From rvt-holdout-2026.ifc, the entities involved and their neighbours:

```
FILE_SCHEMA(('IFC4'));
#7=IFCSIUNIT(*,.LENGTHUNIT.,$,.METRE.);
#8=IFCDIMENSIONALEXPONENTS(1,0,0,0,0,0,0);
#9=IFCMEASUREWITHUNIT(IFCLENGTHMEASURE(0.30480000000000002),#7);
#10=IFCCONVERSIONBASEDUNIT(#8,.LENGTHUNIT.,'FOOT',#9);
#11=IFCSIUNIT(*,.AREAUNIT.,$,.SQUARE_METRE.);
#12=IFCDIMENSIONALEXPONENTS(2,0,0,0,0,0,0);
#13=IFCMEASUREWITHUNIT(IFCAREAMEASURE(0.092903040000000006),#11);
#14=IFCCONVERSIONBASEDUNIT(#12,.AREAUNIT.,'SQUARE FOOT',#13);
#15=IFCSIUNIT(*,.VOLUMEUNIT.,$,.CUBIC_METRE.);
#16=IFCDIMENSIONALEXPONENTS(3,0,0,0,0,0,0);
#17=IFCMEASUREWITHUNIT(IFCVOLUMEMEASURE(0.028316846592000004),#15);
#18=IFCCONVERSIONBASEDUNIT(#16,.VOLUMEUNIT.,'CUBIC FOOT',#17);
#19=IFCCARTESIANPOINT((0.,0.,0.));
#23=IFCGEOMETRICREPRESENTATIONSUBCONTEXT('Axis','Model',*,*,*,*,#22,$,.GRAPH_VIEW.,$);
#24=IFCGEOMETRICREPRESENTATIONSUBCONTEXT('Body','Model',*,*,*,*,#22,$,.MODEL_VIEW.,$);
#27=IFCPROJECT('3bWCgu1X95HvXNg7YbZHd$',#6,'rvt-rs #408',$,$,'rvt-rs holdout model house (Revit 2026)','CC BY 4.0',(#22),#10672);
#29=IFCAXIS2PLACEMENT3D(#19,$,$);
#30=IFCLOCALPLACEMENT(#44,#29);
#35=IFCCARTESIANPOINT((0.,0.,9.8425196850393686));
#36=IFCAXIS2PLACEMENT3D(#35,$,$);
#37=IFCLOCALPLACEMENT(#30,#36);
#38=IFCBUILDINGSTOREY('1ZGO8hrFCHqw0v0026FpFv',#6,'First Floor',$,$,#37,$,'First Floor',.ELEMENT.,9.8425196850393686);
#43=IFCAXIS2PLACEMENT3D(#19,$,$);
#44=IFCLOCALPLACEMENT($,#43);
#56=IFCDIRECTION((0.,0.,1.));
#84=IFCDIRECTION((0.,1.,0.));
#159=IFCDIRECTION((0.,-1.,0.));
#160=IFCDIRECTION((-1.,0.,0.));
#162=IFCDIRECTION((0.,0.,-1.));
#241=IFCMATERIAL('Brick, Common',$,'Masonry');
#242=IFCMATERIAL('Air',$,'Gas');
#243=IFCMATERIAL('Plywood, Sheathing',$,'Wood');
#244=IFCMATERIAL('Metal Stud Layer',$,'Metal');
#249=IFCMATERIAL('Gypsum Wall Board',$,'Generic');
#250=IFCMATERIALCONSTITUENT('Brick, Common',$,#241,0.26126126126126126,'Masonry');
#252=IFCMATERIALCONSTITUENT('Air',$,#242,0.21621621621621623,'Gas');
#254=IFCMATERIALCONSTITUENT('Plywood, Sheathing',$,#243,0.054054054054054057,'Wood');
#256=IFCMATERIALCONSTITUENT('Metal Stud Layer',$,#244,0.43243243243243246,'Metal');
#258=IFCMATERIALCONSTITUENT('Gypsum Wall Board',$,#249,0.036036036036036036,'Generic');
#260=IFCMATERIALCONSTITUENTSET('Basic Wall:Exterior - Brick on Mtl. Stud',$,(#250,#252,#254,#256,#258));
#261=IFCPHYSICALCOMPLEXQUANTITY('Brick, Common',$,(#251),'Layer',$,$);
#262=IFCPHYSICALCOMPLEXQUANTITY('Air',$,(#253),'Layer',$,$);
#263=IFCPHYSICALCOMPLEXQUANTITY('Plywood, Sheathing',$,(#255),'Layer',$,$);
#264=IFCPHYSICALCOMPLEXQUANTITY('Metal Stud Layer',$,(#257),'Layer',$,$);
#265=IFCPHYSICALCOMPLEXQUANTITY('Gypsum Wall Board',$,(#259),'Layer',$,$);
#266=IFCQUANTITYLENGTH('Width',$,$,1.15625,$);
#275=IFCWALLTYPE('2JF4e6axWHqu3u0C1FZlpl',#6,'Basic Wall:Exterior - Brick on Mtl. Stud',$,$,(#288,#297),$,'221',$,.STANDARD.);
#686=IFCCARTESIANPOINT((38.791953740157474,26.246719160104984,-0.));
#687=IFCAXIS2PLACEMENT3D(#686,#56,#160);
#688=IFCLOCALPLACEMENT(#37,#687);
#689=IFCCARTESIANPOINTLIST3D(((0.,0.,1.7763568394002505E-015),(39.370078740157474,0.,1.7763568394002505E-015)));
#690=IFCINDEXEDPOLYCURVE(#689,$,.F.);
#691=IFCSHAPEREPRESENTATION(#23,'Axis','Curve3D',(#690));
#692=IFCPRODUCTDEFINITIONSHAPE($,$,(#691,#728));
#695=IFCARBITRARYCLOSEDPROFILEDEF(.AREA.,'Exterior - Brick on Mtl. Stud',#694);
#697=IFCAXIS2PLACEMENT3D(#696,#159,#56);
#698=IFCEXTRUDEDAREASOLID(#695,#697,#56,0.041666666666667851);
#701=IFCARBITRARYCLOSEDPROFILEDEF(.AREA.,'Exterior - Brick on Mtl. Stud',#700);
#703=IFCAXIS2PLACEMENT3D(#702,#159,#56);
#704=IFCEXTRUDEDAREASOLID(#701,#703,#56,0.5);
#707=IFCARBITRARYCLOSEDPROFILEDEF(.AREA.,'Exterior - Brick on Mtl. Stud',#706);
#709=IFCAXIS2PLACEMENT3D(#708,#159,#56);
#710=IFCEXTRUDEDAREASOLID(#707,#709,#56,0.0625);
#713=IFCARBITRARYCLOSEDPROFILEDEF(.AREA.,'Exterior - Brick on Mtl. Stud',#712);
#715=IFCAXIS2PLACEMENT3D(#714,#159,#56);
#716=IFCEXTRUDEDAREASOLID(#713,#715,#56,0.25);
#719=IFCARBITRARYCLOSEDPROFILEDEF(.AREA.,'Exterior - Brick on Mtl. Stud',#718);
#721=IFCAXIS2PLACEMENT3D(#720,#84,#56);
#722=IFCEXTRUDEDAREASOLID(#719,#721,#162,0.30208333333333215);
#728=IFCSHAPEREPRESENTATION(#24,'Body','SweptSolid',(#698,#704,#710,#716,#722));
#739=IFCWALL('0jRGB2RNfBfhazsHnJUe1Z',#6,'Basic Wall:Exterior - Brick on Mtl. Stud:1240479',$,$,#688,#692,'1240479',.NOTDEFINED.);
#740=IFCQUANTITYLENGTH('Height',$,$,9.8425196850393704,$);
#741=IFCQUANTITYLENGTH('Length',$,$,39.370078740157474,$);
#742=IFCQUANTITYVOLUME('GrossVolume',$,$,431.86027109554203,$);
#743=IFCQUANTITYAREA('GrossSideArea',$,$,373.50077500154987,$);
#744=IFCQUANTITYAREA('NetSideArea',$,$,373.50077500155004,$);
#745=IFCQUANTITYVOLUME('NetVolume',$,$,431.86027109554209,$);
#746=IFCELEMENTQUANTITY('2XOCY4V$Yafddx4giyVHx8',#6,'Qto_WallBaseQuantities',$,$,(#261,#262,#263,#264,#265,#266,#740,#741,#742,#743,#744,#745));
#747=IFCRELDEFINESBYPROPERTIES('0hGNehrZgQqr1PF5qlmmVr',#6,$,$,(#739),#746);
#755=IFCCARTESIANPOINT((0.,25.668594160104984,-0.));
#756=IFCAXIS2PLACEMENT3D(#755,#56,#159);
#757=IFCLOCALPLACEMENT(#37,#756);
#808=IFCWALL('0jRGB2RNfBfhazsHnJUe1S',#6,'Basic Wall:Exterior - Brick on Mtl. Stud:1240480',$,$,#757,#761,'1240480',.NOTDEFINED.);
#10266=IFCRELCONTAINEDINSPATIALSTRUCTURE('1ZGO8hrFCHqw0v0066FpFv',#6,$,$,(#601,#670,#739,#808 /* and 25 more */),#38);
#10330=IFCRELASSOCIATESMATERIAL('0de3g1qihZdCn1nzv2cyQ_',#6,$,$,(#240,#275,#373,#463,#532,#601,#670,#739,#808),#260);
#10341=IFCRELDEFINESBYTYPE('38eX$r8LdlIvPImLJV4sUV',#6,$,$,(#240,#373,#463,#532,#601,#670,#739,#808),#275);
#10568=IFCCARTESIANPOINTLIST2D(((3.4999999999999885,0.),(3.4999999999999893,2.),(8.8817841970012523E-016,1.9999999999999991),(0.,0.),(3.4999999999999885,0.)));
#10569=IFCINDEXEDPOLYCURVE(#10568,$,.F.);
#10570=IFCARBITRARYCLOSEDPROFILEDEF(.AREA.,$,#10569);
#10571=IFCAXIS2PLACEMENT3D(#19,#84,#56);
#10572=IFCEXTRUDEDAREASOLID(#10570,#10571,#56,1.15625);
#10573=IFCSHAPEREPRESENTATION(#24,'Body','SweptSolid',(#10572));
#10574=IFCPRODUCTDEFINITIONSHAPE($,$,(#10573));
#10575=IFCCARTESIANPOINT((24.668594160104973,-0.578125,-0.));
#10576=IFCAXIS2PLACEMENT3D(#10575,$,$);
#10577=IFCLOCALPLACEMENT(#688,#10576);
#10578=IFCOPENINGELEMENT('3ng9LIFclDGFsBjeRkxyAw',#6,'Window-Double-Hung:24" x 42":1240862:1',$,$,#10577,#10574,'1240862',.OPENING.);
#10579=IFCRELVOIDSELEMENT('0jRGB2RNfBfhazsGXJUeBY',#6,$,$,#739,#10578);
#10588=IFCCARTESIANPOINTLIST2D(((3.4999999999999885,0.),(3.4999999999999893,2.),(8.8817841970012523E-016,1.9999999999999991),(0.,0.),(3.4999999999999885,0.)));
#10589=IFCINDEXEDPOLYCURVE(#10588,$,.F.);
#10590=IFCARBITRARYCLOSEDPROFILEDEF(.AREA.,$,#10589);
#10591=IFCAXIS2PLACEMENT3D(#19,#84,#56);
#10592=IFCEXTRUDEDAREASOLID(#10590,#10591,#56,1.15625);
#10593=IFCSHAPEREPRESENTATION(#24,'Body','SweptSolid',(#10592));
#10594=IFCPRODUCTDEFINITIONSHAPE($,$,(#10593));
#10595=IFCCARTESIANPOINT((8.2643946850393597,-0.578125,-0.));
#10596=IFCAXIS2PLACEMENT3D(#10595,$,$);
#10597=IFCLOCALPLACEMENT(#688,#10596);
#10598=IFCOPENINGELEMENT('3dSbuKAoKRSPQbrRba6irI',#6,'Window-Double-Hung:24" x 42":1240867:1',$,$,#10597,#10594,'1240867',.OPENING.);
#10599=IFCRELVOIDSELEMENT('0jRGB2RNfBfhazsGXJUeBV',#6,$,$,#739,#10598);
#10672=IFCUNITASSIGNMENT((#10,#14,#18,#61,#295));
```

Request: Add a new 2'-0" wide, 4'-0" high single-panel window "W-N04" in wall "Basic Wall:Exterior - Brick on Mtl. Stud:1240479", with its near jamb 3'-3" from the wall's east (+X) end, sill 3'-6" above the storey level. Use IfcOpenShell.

```python
import numpy as np
import ifcopenshell
import ifcopenshell.api.feature
import ifcopenshell.api.geometry
import ifcopenshell.api.pset
import ifcopenshell.api.root
import ifcopenshell.api.spatial
import ifcopenshell.geom
import ifcopenshell.util.element
import ifcopenshell.util.placement
import ifcopenshell.util.representation
import ifcopenshell.util.shape
import ifcopenshell.util.unit

model = ifcopenshell.open("rvt-holdout-2026.ifc")
unit_scale = ifcopenshell.util.unit.calculate_unit_scale(model)
area_scale = ifcopenshell.util.unit.calculate_unit_scale(model, "AREAUNIT")
volume_scale = ifcopenshell.util.unit.calculate_unit_scale(model, "VOLUMEUNIT")
settings = ifcopenshell.geom.settings()


def volume(element):
    """Net volume in cubic metres, openings subtracted."""
    shape = ifcopenshell.geom.create_shape(settings, element)
    return ifcopenshell.util.shape.get_volume(shape.geometry)


wall = model.by_guid("0jRGB2RNfBfhazsHnJUe1Z")
storey = ifcopenshell.util.element.get_container(wall, ifc_class="IfcBuildingStorey")
context = ifcopenshell.util.representation.get_context(model, "Model", "Body", "MODEL_VIEW")
before = volume(wall)

width, height, from_end, sill = 0.6096, 1.2192, 0.9906, 1.0668  # metres

# The wall runs along its own X axis, and the end named is its -X end.
wall_shape = ifcopenshell.geom.create_shape(settings, wall)
x, y, z = ifcopenshell.util.shape.get_vertices(wall_shape.geometry).T
start = x.min() + from_end
face, thickness = float(y.min()), float(y.max() - y.min())
wall_matrix = ifcopenshell.util.placement.get_local_placement(wall.ObjectPlacement)
level = ifcopenshell.util.placement.get_local_placement(storey.ObjectPlacement)[2, 3]


def in_wall(x, y):
    """Placement at x, y metres in the wall's axes, at sill height."""
    matrix = wall_matrix.copy()
    matrix[:, 3] = wall_matrix @ np.array([x / unit_scale, y / unit_scale, 0.0, 1.0])
    matrix[2, 3] = level + sill / unit_scale
    return matrix


# Opening: a box that overshoots both wall faces by 50 mm.
opening = ifcopenshell.api.root.create_entity(model, ifc_class="IfcOpeningElement", predefined_type="OPENING")
box = ifcopenshell.api.geometry.add_wall_representation(
    model, context=context, length=width, height=height, thickness=thickness + 0.1
)
ifcopenshell.api.geometry.assign_representation(model, product=opening, representation=box)
ifcopenshell.api.geometry.edit_object_placement(model, product=opening, matrix=in_wall(start, face - 0.05), is_si=False)
ifcopenshell.api.feature.add_feature(model, feature=opening, element=wall)

window = ifcopenshell.api.root.create_entity(model, ifc_class="IfcWindow", name="W-N04", predefined_type="WINDOW")
window.OverallWidth, window.OverallHeight = width / unit_scale, height / unit_scale
window.PartitioningType = "SINGLE_PANEL"
body = ifcopenshell.api.geometry.add_window_representation(
    model,
    context=context,
    overall_width=window.OverallWidth,
    overall_height=window.OverallHeight,
    partition_type="SINGLE_PANEL",
)
ifcopenshell.api.geometry.assign_representation(model, product=window, representation=body)
ifcopenshell.api.spatial.assign_container(model, products=[window], relating_structure=storey)
ifcopenshell.api.feature.add_filling(model, opening=opening, element=window)

# Centre the window in the wall's thickness.
ifcopenshell.api.geometry.edit_object_placement(model, product=window, matrix=in_wall(start, face), is_si=False)
window_shape = ifcopenshell.geom.create_shape(settings, window)
depth = ifcopenshell.util.shape.get_vertices(window_shape.geometry)[:, 1]
offset = face + thickness / 2 - (depth.min() + depth.max()) / 2
ifcopenshell.api.geometry.edit_object_placement(model, product=window, matrix=in_wall(start, offset), is_si=False)

after = volume(wall)

# Update the wall's stored quantities.
qto = model.by_id(ifcopenshell.util.element.get_pset(wall, "Qto_WallBaseQuantities", should_inherit=False)["id"])
ifcopenshell.api.pset.edit_qto(model, qto=qto, properties={
    "NetSideArea": after / thickness / area_scale,
    "NetVolume": after / volume_scale,
})

print(f"wall volume {before:.3f} -> {after:.3f} m3")

model.write("rvt-holdout-2026_edited.ifc")
```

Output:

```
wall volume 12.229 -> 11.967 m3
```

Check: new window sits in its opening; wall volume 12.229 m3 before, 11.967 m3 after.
